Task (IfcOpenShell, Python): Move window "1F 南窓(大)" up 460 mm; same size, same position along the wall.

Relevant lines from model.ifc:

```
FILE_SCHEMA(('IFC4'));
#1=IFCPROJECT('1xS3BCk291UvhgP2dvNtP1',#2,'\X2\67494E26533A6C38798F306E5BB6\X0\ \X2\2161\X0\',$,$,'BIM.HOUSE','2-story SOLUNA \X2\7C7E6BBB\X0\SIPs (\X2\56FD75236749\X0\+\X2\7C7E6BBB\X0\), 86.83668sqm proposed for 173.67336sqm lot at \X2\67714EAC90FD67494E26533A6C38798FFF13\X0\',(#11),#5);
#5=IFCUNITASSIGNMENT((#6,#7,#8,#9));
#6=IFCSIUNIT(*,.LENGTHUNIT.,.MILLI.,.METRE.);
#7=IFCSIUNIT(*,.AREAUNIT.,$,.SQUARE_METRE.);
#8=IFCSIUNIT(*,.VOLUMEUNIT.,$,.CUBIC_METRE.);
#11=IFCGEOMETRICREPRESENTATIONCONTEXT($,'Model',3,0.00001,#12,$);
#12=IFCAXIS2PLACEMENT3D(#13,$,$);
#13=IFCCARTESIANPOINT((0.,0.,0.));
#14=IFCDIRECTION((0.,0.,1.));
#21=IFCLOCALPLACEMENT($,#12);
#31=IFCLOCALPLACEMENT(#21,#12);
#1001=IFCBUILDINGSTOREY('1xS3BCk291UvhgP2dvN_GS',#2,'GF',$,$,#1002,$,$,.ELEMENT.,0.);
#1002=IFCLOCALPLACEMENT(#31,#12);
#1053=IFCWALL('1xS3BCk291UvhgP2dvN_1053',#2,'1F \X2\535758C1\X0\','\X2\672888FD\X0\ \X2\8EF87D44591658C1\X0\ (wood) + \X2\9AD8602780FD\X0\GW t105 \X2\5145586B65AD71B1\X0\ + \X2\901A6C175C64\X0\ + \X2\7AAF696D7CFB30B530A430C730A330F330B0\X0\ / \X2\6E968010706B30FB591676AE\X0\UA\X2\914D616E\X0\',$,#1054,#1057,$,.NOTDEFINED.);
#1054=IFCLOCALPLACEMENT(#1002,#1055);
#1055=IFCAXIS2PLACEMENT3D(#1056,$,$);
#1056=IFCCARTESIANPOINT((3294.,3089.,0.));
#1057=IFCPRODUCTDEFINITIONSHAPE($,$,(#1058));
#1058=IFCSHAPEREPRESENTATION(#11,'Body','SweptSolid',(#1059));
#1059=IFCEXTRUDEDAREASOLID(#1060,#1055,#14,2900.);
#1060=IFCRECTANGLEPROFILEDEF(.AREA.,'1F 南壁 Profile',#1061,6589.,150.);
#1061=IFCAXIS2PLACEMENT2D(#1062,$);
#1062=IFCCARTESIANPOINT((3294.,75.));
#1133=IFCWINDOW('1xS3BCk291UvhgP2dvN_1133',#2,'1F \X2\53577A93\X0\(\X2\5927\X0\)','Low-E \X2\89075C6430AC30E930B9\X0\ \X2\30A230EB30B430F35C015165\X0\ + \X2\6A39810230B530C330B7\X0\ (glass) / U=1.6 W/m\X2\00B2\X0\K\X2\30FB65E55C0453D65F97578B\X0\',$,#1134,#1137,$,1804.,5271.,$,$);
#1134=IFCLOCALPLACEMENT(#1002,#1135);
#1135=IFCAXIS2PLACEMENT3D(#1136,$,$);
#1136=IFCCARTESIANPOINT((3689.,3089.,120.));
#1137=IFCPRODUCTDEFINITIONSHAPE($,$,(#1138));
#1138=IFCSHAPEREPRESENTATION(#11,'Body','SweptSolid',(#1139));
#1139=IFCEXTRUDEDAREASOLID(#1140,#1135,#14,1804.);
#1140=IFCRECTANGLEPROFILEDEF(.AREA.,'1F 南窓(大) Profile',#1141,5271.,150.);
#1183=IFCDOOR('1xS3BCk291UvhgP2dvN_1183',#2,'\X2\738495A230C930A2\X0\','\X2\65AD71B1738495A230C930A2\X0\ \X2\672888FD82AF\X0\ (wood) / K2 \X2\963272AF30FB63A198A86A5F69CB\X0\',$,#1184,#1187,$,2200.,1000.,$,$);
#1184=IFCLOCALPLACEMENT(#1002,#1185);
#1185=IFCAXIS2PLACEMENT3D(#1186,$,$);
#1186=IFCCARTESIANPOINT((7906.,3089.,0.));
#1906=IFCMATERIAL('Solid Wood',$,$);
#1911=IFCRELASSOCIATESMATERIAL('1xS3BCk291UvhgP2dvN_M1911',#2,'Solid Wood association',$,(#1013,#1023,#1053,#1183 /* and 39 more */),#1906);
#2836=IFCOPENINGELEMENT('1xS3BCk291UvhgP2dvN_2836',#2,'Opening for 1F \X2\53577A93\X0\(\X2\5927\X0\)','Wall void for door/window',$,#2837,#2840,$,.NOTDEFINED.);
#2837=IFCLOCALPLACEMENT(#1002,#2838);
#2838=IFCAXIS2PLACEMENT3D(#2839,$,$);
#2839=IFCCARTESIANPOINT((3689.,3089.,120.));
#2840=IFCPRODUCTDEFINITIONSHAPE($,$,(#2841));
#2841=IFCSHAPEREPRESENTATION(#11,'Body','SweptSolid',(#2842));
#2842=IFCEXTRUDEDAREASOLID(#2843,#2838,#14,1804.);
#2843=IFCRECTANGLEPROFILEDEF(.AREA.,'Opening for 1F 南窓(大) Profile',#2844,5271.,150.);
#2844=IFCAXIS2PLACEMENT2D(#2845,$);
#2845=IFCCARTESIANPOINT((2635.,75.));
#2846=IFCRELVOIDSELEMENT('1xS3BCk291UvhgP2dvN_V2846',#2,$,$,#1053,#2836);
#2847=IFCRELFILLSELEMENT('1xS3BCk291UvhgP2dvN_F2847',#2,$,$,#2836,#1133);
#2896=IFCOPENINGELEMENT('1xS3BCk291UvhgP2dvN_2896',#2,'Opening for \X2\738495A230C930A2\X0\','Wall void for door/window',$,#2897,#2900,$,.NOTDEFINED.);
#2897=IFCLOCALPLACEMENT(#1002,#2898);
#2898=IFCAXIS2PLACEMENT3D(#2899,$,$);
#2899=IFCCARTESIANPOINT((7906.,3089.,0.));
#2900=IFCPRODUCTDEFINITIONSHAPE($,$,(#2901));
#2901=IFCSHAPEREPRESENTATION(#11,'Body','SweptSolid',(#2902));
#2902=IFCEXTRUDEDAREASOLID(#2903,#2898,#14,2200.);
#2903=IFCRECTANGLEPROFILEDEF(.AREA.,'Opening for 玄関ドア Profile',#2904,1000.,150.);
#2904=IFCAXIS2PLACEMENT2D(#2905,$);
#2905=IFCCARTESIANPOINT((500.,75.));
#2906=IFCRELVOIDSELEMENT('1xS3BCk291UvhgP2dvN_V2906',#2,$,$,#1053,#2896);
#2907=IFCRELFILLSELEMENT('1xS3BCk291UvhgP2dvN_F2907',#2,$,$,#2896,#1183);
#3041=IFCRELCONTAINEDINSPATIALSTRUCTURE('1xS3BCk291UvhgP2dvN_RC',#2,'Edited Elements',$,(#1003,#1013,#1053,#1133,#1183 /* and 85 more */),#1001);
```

```python
import numpy as np
import ifcopenshell
import ifcopenshell.api.geometry
import ifcopenshell.util.placement
import ifcopenshell.util.unit

model = ifcopenshell.open("model.ifc")
unit_scale = ifcopenshell.util.unit.calculate_unit_scale(model)

window = model.by_guid("1xS3BCk291UvhgP2dvN_1133")
opening = window.FillsVoids[0].RelatingOpeningElement
dz = 0.46 / unit_scale

shift = np.array([0.0, 0.0, dz])
# The window is not placed relative to its opening, so move both.
for product in (opening, window):
    matrix = ifcopenshell.util.placement.get_local_placement(product.ObjectPlacement)
    matrix[:3, 3] += shift
    ifcopenshell.api.geometry.edit_object_placement(model, product=product, matrix=matrix, is_si=False)

print(f"moved by {dz * unit_scale:+.3f} m")

model.write("model_updated.ifc")
```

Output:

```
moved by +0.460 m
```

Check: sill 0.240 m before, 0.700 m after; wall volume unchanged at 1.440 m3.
